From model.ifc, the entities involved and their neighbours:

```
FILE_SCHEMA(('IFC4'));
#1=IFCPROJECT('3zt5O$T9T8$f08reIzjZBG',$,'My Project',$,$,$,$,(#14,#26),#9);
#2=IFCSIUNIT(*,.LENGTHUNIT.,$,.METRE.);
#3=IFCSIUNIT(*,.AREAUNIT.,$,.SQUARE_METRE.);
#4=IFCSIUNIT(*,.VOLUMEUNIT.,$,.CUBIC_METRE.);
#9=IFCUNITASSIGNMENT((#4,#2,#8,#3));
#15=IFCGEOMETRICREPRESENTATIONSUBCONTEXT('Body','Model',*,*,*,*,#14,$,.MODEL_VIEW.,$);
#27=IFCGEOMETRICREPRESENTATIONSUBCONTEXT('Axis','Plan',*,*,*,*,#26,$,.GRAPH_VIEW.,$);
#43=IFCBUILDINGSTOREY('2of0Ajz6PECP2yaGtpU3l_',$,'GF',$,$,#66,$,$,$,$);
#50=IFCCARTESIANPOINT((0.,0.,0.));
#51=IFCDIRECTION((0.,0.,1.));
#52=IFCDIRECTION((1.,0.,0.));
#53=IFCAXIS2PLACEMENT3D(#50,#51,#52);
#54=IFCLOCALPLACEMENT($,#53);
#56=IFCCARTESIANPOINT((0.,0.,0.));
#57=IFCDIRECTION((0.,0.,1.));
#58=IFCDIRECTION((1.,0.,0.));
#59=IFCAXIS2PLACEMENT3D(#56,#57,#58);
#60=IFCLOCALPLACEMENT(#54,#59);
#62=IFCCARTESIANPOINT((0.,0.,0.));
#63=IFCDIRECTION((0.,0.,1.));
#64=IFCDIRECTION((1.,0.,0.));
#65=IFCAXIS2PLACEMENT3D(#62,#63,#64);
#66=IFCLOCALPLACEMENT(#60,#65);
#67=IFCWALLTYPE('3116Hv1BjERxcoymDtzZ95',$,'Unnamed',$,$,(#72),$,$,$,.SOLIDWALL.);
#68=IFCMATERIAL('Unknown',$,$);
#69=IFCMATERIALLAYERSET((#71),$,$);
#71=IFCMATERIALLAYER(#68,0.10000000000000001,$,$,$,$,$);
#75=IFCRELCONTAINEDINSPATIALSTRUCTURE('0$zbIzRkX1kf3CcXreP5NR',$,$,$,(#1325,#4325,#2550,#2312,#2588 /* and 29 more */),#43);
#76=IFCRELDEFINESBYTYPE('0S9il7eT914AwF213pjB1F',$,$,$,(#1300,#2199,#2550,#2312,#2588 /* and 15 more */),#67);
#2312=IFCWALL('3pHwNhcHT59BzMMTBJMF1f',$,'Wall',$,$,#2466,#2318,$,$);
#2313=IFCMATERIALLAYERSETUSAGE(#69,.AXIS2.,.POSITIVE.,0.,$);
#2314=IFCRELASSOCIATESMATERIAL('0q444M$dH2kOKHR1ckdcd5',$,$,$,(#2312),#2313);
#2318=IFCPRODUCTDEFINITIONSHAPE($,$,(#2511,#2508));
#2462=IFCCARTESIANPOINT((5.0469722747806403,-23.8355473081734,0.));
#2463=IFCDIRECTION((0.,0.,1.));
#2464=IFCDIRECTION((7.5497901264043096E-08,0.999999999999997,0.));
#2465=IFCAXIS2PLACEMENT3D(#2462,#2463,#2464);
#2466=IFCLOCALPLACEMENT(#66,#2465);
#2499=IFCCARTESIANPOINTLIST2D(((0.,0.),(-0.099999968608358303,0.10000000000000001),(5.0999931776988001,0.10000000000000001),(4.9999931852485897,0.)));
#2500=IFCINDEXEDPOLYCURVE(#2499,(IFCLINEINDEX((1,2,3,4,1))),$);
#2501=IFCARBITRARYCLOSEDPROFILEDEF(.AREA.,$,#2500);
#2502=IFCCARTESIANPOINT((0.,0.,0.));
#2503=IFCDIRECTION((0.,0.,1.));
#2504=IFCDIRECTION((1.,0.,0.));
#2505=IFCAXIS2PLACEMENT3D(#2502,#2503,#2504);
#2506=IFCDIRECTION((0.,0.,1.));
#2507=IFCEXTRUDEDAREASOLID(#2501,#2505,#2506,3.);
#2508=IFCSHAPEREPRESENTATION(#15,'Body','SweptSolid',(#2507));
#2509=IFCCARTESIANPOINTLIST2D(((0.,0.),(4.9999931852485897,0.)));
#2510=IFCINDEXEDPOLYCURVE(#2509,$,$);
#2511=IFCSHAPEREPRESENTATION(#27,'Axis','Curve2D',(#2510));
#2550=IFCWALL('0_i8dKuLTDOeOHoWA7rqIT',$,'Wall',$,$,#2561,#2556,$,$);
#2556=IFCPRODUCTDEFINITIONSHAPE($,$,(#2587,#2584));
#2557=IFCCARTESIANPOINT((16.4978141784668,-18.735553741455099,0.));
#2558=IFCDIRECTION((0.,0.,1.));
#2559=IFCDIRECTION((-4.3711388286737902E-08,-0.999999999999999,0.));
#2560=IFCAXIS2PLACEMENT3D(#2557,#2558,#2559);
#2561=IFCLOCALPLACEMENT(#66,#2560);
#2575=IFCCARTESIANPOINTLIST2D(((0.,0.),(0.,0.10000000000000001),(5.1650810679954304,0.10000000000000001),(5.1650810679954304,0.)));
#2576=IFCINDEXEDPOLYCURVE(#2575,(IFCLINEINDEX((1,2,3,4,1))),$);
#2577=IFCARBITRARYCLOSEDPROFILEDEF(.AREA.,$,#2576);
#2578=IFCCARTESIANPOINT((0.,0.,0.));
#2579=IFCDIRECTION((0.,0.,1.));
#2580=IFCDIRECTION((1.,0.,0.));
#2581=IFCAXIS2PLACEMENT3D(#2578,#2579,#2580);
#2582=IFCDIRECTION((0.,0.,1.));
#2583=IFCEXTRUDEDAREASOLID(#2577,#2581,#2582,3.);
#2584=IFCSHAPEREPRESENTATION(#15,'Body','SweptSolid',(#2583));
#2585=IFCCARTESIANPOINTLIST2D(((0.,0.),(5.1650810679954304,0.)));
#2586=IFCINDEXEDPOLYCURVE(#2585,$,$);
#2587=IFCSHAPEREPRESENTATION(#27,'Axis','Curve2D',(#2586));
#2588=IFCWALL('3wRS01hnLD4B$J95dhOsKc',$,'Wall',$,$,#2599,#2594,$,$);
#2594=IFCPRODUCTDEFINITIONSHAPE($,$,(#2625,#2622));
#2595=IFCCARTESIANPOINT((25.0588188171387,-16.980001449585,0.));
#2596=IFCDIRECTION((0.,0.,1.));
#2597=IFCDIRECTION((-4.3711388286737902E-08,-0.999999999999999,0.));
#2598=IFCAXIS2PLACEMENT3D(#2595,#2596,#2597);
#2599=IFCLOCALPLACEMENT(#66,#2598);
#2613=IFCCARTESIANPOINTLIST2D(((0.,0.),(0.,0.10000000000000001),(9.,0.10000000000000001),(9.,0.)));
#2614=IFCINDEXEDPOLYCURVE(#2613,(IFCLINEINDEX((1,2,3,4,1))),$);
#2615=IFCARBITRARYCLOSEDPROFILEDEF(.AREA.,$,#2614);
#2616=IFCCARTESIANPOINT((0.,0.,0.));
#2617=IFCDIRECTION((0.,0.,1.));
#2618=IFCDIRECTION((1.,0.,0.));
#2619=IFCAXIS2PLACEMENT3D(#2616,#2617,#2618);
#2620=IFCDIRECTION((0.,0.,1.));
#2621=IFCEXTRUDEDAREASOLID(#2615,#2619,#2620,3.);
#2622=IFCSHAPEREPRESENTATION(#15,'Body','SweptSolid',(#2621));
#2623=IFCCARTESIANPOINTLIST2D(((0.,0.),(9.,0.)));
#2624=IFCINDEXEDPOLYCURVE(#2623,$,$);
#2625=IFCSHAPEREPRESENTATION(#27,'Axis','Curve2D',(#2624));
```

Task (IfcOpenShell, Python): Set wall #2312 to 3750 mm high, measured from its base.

```python
import ifcopenshell
import ifcopenshell.geom
import ifcopenshell.util.representation
import ifcopenshell.util.shape
import ifcopenshell.util.unit

model = ifcopenshell.open("model.ifc")
unit_scale = ifcopenshell.util.unit.calculate_unit_scale(model)
settings = ifcopenshell.geom.settings()


def volume(element):
    """Net volume in cubic metres, openings subtracted."""
    shape = ifcopenshell.geom.create_shape(settings, element)
    return ifcopenshell.util.shape.get_volume(shape.geometry)


wall = model.by_id(2312)
before = volume(wall)

body = ifcopenshell.util.representation.get_representation(wall, "Model", "Body")
solid = body.Items[0]
old_height = solid.Depth
solid.Depth = 3.75 / unit_scale
after = volume(wall)

print(f"height {old_height:g} -> {solid.Depth:g}, volume {before:.3f} -> {after:.3f} m3")

model.write("model_updated.ifc")
```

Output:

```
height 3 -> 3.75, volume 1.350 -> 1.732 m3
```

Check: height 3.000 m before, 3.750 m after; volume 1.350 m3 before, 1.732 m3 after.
